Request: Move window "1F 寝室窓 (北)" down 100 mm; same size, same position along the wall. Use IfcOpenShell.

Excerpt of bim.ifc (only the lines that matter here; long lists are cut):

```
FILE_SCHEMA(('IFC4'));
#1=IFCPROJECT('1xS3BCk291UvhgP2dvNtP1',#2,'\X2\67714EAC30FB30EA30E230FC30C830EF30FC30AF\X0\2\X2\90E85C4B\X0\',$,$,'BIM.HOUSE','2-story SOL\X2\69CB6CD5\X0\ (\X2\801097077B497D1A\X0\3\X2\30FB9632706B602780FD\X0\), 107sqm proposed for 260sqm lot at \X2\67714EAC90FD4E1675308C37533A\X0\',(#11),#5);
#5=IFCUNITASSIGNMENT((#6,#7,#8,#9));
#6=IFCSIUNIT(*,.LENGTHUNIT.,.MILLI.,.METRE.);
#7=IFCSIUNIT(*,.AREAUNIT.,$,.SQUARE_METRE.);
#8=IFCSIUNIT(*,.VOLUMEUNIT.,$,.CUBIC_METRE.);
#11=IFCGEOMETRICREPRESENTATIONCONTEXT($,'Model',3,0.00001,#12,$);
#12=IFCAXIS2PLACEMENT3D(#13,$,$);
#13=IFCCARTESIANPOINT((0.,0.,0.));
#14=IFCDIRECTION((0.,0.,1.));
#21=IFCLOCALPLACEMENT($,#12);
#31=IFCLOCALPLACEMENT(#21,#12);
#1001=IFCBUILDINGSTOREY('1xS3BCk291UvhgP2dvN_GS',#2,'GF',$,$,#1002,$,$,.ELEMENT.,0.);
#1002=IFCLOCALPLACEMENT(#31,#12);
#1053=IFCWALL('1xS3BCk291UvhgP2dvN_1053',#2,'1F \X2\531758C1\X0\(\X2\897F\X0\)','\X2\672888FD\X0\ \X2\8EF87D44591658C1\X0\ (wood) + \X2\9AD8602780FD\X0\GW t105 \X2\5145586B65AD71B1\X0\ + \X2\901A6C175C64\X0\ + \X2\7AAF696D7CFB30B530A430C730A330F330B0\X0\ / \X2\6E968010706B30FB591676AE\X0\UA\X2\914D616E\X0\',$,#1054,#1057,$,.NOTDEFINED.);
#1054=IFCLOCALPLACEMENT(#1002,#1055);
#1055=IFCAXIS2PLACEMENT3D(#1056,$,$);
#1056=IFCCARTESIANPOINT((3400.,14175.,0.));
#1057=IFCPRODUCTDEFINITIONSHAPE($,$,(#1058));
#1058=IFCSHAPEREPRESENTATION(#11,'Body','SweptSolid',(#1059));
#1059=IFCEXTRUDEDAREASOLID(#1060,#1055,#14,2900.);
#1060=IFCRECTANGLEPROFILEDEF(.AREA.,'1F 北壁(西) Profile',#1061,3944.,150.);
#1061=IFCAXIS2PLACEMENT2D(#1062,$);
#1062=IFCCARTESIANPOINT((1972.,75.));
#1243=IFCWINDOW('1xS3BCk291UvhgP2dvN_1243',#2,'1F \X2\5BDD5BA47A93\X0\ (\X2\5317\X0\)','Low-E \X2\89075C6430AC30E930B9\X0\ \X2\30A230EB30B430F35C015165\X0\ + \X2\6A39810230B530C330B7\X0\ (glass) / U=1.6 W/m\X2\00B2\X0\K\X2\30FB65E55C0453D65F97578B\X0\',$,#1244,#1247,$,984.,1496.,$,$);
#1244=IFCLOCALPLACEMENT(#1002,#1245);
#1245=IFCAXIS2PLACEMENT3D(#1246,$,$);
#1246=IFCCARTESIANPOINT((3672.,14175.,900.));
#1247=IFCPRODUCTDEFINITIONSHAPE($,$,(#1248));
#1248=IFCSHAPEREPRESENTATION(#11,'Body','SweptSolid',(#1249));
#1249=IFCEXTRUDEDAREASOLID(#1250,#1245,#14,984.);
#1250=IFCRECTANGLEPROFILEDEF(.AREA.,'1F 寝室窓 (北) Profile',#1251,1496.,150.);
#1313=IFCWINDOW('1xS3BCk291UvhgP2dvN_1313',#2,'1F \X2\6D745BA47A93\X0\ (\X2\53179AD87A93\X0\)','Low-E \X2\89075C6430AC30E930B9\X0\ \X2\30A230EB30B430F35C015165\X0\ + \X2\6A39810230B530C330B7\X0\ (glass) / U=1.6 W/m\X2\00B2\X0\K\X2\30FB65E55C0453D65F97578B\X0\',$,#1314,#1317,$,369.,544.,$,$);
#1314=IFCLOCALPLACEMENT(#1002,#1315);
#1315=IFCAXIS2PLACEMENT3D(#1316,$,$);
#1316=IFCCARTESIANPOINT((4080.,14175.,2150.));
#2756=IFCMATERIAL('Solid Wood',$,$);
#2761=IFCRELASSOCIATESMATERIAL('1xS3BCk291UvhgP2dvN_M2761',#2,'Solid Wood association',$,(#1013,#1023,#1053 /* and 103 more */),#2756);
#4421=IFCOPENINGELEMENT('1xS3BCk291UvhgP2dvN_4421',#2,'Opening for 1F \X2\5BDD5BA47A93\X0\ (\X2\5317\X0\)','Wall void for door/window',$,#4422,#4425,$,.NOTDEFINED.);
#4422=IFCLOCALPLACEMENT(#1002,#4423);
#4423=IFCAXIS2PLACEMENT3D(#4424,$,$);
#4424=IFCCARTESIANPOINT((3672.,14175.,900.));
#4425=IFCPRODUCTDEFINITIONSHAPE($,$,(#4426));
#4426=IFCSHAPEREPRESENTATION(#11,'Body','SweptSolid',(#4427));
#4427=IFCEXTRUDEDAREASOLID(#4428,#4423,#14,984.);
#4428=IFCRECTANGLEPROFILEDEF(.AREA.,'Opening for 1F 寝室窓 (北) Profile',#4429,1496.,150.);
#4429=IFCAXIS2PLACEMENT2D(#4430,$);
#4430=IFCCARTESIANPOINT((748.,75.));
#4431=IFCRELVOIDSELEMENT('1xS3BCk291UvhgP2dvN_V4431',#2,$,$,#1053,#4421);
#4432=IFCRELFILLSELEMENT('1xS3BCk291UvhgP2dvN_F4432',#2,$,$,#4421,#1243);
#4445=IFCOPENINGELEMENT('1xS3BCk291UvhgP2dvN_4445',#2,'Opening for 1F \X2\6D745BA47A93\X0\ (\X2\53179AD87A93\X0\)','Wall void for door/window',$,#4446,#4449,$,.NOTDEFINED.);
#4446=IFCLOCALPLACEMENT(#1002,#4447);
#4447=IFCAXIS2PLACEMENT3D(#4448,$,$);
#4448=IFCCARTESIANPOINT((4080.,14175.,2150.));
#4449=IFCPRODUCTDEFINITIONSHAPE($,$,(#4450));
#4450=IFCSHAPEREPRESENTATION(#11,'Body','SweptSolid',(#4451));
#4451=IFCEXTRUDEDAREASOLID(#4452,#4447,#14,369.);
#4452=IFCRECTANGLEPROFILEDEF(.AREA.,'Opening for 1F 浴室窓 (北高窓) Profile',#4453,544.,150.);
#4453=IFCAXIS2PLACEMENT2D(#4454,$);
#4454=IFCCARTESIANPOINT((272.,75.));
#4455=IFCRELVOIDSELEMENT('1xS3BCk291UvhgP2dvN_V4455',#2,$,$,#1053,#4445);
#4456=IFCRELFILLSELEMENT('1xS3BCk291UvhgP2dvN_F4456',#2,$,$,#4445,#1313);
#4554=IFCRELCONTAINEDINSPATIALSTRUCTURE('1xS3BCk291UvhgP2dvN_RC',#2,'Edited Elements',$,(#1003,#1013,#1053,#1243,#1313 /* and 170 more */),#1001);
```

```python
import numpy as np
import ifcopenshell
import ifcopenshell.api.geometry
import ifcopenshell.util.placement
import ifcopenshell.util.unit

model = ifcopenshell.open("bim.ifc")
unit_scale = ifcopenshell.util.unit.calculate_unit_scale(model)

window = model.by_guid("1xS3BCk291UvhgP2dvN_1243")
opening = window.FillsVoids[0].RelatingOpeningElement
dz = -100.0

shift = np.array([0.0, 0.0, dz])
# The window is not placed relative to its opening, so move both.
for product in (opening, window):
    matrix = ifcopenshell.util.placement.get_local_placement(product.ObjectPlacement)
    matrix[:3, 3] += shift
    ifcopenshell.api.geometry.edit_object_placement(model, product=product, matrix=matrix, is_si=False)

print(f"moved by {dz * unit_scale:+.3f} m")

model.write("bim_rev.ifc")
```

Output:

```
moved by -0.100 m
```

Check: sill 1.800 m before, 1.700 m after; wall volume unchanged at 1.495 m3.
